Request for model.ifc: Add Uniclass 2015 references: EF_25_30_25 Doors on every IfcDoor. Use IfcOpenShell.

First a look at what the model holds.

```python
import ifcopenshell

model = ifcopenshell.open("model.ifc")
print(model.schema)
print("classifications:", [c.Name for c in model.by_type("IfcClassification")])
for ifc_class in ("IfcDoor", "IfcRoof", "IfcStair", "IfcWall", "IfcWindow"):
    print(ifc_class, len(model.by_type(ifc_class)))
```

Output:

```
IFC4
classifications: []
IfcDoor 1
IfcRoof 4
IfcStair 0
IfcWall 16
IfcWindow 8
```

```python
import ifcopenshell
import ifcopenshell.api.classification

model = ifcopenshell.open("model.ifc")

system = ifcopenshell.api.classification.add_classification(model, classification="Uniclass 2015")

codes = {
    "IfcDoor": ("EF_25_30_25", "Doors"),
}
for ifc_class, (code, name) in codes.items():
    products = model.by_type(ifc_class)
    ifcopenshell.api.classification.add_reference(
        model, products=products, classification=system, identification=code, name=name
    )
    print(code, len(products))

model.write("model_rev.ifc")
```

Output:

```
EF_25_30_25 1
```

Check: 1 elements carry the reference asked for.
